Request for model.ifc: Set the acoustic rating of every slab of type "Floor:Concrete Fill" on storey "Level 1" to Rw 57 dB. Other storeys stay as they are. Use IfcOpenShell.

First a look at what the model holds.

```python
import ifcopenshell
import ifcopenshell.util.element

model = ifcopenshell.open("model.ifc")
print(model.schema)
storey = next(s for s in model.by_type("IfcBuildingStorey") if s.Name == "Level 1")
slabs = [e for e in ifcopenshell.util.element.get_decomposition(storey) if e.is_a("IfcSlab")]
seen = {}
for e in slabs:
    element_type = ifcopenshell.util.element.get_type(e)
    key = (element_type.Name if element_type != e and element_type else None, ifcopenshell.util.element.get_pset(e, "Pset_SlabCommon", "AcousticRating"))
    seen[key] = seen.get(key, 0) + 1
for (name, value), count in sorted(seen.items(), key=str):
    print(count, "x", name, "|", value)
```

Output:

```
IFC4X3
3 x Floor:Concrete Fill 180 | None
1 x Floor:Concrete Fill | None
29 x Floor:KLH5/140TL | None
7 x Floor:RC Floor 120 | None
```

```python
import ifcopenshell
import ifcopenshell.api.pset
import ifcopenshell.util.element

model = ifcopenshell.open("model.ifc")

storey = next(s for s in model.by_type("IfcBuildingStorey") if s.Name == "Level 1")
slabs = [e for e in ifcopenshell.util.element.get_decomposition(storey) if e.is_a("IfcSlab")]

count = 0
for e in slabs:
    element_type = ifcopenshell.util.element.get_type(e)
    if element_type in (None, e) or element_type.Name != "Floor:Concrete Fill":
        continue
    # add_pset returns the element's existing set when there is one.
    pset = ifcopenshell.api.pset.add_pset(model, product=e, name="Pset_SlabCommon")
    ifcopenshell.api.pset.edit_pset(model, pset=pset, properties={"AcousticRating": "Rw 57 dB"})
    count += 1

print(count, "slabs updated")

model.write("model_v2.ifc")
```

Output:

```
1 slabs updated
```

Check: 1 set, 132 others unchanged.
